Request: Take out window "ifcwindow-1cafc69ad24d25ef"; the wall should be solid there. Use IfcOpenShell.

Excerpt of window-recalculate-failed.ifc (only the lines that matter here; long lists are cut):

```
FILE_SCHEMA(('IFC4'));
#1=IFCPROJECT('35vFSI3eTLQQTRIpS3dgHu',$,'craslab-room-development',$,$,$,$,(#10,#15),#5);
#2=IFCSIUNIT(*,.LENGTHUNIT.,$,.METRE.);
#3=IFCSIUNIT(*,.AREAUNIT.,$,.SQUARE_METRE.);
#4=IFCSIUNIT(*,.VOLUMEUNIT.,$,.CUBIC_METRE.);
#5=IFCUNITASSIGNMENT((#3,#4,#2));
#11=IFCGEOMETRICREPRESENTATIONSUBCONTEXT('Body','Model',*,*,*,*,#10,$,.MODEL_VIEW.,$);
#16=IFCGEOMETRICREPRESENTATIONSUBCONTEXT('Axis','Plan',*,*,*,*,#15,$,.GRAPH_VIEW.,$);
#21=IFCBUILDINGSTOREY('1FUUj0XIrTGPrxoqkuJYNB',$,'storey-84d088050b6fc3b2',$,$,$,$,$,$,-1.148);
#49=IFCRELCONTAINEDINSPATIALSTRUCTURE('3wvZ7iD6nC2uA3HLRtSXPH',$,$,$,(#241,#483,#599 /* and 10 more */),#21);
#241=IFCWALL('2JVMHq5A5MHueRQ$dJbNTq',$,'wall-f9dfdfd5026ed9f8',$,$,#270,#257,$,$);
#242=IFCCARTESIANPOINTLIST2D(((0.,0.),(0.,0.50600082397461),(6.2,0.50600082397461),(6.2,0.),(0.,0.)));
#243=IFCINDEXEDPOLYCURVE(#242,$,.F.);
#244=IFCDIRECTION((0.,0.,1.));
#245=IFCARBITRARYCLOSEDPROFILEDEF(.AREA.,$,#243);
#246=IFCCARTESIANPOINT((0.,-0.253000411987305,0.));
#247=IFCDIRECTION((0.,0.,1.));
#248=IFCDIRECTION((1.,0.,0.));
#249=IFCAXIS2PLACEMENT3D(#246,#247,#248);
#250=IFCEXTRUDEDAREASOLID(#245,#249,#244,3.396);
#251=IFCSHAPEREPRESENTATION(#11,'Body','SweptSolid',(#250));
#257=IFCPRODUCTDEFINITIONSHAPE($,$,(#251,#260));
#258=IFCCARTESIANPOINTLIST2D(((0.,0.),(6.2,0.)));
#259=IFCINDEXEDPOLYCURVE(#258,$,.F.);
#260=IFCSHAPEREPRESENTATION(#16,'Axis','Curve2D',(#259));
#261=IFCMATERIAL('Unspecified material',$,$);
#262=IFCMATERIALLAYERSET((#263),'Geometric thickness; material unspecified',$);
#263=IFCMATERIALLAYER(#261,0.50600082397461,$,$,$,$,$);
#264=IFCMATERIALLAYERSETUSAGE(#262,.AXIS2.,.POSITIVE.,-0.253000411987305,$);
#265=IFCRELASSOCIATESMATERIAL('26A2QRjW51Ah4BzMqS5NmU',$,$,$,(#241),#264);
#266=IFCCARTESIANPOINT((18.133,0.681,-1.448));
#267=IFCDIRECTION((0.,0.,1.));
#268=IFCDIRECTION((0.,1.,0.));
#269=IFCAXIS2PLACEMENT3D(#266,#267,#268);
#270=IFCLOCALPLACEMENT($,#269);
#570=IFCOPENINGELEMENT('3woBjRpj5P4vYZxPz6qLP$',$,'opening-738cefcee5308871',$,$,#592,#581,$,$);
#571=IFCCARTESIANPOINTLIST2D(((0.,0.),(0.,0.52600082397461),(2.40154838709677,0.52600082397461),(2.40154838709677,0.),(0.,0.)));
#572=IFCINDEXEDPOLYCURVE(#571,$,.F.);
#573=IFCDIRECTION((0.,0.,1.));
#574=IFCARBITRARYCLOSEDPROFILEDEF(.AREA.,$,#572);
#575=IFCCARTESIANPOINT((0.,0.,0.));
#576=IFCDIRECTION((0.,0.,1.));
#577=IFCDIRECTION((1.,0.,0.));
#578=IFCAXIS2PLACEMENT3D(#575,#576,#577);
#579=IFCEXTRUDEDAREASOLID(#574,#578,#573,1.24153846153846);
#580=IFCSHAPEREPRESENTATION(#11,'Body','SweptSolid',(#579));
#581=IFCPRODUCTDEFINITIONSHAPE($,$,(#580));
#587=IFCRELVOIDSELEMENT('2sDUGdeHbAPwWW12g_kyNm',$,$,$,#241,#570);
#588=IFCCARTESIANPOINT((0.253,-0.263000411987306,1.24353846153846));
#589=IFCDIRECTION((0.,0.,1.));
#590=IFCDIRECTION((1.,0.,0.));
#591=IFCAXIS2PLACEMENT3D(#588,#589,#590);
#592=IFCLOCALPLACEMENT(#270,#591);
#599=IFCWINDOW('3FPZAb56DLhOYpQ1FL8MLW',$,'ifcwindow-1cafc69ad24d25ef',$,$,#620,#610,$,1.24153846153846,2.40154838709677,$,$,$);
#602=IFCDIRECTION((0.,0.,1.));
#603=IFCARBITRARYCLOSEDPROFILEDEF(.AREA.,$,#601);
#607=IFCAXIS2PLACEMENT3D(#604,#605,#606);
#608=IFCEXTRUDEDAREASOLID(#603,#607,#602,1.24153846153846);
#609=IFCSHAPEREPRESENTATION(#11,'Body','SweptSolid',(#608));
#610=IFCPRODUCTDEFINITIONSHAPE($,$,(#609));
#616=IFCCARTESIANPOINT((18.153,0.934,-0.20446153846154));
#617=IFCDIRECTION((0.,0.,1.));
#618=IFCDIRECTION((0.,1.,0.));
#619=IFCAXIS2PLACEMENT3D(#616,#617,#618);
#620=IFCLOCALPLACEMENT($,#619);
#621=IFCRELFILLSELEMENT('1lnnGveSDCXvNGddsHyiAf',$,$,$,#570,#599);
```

```python
import ifcopenshell
import ifcopenshell.api.feature
import ifcopenshell.api.root
import ifcopenshell.geom
import ifcopenshell.util.shape

model = ifcopenshell.open("window-recalculate-failed.ifc")
settings = ifcopenshell.geom.settings()


def volume(element):
    """Net volume in cubic metres, openings subtracted."""
    shape = ifcopenshell.geom.create_shape(settings, element)
    return ifcopenshell.util.shape.get_volume(shape.geometry)


window = model.by_guid("3FPZAb56DLhOYpQ1FL8MLW")
opening = window.FillsVoids[0].RelatingOpeningElement
wall = opening.VoidsElements[0].RelatingBuildingElement
before = volume(wall)

ifcopenshell.api.root.remove_product(model, product=window)
ifcopenshell.api.feature.remove_feature(model, feature=opening)

after = volume(wall)

print(f"wall volume {before:.3f} -> {after:.3f} m3")

model.write("window-recalculate-failed_v2.ifc")
```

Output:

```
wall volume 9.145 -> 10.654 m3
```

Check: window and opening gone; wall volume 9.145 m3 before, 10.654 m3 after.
